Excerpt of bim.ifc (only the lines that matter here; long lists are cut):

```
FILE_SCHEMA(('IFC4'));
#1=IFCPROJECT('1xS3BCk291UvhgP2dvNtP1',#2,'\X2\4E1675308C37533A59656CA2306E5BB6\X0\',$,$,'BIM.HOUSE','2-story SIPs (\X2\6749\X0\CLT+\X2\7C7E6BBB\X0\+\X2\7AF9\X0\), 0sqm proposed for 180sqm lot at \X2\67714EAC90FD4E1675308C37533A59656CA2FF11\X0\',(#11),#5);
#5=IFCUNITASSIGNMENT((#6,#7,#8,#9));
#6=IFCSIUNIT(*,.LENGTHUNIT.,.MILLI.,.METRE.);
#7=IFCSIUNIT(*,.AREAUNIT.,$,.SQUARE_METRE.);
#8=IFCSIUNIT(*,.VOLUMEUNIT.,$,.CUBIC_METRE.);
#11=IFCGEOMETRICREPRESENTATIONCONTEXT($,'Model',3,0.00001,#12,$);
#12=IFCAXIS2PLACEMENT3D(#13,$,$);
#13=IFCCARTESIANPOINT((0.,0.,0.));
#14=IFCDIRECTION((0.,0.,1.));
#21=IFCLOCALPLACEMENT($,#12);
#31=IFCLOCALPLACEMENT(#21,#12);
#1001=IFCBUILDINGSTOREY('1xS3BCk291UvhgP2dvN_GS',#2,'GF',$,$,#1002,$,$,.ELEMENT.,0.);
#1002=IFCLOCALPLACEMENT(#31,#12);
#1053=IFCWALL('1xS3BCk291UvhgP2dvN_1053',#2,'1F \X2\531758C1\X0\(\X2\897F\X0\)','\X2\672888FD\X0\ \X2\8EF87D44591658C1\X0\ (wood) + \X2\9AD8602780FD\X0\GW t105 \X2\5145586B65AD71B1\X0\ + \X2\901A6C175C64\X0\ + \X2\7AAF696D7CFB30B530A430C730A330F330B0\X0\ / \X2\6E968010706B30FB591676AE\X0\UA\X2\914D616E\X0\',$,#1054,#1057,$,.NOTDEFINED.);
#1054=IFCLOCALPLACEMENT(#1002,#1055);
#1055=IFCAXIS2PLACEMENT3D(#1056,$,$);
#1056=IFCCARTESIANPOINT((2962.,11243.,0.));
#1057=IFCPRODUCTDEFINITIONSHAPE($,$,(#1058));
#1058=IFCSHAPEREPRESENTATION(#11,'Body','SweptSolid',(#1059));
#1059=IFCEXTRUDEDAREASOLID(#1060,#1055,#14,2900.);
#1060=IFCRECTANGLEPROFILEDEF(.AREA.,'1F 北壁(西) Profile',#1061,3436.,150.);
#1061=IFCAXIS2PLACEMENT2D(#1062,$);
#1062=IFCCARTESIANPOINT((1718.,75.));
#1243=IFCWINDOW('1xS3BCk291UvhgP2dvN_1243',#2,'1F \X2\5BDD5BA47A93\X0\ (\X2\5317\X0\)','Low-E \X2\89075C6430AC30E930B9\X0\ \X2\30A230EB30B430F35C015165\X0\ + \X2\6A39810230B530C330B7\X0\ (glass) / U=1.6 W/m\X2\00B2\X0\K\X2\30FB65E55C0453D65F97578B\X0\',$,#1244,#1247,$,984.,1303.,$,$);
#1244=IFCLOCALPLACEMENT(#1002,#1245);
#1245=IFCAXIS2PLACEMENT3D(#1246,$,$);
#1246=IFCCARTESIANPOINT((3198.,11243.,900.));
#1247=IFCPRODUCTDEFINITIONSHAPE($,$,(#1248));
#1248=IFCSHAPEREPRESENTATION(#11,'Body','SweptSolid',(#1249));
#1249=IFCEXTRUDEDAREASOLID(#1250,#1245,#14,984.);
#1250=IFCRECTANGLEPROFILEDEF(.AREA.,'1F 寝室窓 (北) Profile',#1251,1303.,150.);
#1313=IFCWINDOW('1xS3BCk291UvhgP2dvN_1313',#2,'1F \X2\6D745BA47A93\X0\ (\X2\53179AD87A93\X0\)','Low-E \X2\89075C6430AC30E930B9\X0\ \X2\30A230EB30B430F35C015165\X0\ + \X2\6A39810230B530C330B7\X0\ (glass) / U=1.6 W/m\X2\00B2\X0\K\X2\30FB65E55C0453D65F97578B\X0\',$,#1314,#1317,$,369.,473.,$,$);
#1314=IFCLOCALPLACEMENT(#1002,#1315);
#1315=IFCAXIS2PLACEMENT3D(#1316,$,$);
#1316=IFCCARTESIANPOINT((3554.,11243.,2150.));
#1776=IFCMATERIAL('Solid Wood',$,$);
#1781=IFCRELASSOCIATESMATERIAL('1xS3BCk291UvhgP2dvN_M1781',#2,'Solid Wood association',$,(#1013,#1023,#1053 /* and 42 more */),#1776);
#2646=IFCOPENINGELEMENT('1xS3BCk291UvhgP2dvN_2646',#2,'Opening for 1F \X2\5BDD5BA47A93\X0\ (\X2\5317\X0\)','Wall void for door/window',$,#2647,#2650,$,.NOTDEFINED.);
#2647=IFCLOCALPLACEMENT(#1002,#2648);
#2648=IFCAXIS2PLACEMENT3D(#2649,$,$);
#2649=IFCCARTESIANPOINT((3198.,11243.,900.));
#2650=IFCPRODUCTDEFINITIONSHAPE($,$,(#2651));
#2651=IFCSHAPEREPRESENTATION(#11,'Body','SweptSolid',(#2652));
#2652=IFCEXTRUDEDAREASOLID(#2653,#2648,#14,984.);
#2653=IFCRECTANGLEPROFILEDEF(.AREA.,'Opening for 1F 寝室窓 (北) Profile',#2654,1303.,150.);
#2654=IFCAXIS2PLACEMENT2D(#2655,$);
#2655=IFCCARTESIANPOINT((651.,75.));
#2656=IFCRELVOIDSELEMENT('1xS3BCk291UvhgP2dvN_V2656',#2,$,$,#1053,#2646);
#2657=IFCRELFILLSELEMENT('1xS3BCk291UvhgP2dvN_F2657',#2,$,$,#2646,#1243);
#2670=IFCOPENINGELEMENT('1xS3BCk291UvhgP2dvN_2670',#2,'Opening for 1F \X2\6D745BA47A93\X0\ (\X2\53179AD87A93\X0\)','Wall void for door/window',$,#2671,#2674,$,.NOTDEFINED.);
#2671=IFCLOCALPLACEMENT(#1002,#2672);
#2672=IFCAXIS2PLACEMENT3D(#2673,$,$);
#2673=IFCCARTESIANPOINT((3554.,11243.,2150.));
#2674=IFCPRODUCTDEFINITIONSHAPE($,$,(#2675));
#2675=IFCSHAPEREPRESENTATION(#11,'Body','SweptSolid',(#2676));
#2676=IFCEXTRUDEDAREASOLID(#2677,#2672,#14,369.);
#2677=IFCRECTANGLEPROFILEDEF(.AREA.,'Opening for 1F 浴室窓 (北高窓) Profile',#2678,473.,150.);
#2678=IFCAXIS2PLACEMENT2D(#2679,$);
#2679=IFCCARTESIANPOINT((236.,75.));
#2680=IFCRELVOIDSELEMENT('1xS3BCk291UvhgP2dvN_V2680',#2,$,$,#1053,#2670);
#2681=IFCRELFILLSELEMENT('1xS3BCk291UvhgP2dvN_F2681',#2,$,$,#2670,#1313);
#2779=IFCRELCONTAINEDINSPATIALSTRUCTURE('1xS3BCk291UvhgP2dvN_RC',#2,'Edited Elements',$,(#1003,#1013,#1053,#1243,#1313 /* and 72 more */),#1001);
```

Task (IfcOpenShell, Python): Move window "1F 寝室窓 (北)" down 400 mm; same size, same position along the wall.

```python
import numpy as np
import ifcopenshell
import ifcopenshell.api.geometry
import ifcopenshell.util.placement
import ifcopenshell.util.unit

model = ifcopenshell.open("bim.ifc")
unit_scale = ifcopenshell.util.unit.calculate_unit_scale(model)

window = model.by_guid("1xS3BCk291UvhgP2dvN_1243")
opening = window.FillsVoids[0].RelatingOpeningElement
dz = -0.4 / unit_scale

shift = np.array([0.0, 0.0, dz])
# The window is not placed relative to its opening, so move both.
for product in (opening, window):
    matrix = ifcopenshell.util.placement.get_local_placement(product.ObjectPlacement)
    matrix[:3, 3] += shift
    ifcopenshell.api.geometry.edit_object_placement(model, product=product, matrix=matrix, is_si=False)

print(f"moved by {dz * unit_scale:+.3f} m")

model.write("bim_rev.ifc")
```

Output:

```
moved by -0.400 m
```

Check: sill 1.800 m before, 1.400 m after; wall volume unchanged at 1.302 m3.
